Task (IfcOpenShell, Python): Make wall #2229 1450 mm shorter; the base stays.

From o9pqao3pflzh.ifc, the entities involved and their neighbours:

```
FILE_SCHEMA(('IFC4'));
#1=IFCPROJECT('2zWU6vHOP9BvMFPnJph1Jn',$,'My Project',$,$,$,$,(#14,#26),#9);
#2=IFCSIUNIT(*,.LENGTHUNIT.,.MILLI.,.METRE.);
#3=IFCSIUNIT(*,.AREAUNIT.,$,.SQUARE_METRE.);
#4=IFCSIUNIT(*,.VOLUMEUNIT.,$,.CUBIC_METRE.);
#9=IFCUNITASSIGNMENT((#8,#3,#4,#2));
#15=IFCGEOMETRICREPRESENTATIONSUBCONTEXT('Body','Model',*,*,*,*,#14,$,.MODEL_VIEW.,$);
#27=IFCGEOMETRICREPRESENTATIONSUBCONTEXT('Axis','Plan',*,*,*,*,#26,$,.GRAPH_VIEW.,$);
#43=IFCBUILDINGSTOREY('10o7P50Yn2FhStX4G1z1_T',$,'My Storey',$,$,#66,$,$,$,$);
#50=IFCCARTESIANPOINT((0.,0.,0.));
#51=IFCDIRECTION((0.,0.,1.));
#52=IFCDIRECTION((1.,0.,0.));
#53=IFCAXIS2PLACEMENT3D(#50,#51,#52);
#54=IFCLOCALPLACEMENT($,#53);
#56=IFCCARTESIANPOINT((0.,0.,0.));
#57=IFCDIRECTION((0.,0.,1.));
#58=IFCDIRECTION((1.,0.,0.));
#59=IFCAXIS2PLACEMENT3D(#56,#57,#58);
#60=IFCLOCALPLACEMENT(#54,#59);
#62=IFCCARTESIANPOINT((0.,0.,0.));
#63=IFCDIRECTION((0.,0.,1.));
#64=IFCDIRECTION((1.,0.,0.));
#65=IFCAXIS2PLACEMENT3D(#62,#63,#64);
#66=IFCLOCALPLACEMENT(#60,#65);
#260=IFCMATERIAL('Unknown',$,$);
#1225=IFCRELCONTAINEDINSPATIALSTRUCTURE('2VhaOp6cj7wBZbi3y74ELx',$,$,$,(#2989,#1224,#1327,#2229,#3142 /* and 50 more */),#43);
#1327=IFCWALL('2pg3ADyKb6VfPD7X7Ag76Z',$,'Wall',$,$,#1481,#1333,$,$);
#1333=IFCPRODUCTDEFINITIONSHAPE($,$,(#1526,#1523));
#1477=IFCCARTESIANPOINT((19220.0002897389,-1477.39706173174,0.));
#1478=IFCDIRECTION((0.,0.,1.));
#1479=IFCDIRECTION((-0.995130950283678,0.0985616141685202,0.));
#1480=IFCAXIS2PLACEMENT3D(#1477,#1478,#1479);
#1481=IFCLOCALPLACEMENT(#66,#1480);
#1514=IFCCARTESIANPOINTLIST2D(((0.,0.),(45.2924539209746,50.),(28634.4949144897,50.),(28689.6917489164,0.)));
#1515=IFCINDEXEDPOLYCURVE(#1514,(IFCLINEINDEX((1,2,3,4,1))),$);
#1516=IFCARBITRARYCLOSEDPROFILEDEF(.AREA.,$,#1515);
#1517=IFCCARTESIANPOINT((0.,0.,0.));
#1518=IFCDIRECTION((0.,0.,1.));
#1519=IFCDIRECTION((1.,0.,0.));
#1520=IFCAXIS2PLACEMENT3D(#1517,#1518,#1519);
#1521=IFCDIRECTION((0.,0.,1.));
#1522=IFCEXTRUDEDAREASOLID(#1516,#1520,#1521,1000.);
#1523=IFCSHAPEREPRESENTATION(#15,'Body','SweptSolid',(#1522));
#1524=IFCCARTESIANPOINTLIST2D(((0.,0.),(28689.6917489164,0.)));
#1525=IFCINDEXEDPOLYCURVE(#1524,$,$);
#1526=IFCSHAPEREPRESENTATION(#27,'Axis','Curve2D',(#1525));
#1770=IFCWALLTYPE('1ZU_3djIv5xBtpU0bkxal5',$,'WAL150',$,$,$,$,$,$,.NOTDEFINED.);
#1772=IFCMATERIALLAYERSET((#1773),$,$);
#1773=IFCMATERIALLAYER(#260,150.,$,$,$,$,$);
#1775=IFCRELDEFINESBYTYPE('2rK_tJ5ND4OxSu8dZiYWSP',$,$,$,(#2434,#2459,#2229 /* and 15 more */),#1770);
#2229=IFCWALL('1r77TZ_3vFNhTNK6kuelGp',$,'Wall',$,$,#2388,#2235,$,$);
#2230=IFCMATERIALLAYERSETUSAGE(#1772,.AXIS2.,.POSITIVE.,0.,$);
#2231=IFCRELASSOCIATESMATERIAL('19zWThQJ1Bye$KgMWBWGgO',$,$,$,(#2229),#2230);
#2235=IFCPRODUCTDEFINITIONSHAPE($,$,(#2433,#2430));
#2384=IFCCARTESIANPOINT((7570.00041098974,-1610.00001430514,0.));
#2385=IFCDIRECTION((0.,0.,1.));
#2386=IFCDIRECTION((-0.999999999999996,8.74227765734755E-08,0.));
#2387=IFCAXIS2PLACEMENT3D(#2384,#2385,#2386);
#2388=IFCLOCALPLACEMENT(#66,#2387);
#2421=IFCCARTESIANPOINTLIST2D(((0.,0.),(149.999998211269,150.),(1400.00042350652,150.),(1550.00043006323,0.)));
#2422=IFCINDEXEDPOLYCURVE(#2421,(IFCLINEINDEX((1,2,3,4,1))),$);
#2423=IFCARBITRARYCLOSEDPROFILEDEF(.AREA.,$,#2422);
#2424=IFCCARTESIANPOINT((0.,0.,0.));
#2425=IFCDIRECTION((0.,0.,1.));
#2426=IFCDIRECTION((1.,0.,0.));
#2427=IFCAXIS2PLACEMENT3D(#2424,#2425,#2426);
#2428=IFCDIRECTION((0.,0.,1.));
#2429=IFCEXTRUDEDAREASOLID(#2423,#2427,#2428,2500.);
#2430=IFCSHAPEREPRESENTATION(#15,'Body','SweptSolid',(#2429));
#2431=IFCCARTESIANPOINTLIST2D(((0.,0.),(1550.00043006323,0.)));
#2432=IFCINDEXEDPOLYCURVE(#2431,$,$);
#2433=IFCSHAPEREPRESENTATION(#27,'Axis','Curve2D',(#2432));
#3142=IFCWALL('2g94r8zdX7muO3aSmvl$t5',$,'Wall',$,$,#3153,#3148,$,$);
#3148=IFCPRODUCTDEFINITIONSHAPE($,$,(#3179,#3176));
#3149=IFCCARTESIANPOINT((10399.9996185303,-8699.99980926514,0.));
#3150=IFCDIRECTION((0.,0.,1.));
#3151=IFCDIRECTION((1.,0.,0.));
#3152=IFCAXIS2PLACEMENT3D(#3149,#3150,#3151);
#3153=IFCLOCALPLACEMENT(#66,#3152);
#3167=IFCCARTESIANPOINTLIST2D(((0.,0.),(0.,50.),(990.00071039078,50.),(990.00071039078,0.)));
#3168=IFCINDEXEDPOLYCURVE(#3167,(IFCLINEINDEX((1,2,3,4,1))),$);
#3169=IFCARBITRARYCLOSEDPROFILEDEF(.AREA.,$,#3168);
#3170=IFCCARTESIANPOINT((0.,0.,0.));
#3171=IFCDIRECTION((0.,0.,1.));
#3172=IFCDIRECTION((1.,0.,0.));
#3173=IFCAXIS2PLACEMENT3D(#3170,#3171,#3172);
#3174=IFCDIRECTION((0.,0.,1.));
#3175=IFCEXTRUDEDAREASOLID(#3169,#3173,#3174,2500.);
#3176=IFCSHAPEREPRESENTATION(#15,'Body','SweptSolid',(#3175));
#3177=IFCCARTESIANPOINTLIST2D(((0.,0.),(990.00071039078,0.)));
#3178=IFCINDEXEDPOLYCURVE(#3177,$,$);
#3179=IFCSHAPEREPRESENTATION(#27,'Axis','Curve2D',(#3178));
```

```python
import ifcopenshell
import ifcopenshell.geom
import ifcopenshell.util.representation
import ifcopenshell.util.shape
import ifcopenshell.util.unit

model = ifcopenshell.open("o9pqao3pflzh.ifc")
unit_scale = ifcopenshell.util.unit.calculate_unit_scale(model)
settings = ifcopenshell.geom.settings()


def volume(element):
    """Net volume in cubic metres, openings subtracted."""
    shape = ifcopenshell.geom.create_shape(settings, element)
    return ifcopenshell.util.shape.get_volume(shape.geometry)


wall = model.by_guid("1r77TZ_3vFNhTNK6kuelGp")
before = volume(wall)

body = ifcopenshell.util.representation.get_representation(wall, "Model", "Body")
solid = body.Items[0]
old_height = solid.Depth
solid.Depth -= 1.45 / unit_scale
after = volume(wall)

print(f"height {old_height:g} -> {solid.Depth:g}, volume {before:.3f} -> {after:.3f} m3")

model.write("o9pqao3pflzh_updated.ifc")
```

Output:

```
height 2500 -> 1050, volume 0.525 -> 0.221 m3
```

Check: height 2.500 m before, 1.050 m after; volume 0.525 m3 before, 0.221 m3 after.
